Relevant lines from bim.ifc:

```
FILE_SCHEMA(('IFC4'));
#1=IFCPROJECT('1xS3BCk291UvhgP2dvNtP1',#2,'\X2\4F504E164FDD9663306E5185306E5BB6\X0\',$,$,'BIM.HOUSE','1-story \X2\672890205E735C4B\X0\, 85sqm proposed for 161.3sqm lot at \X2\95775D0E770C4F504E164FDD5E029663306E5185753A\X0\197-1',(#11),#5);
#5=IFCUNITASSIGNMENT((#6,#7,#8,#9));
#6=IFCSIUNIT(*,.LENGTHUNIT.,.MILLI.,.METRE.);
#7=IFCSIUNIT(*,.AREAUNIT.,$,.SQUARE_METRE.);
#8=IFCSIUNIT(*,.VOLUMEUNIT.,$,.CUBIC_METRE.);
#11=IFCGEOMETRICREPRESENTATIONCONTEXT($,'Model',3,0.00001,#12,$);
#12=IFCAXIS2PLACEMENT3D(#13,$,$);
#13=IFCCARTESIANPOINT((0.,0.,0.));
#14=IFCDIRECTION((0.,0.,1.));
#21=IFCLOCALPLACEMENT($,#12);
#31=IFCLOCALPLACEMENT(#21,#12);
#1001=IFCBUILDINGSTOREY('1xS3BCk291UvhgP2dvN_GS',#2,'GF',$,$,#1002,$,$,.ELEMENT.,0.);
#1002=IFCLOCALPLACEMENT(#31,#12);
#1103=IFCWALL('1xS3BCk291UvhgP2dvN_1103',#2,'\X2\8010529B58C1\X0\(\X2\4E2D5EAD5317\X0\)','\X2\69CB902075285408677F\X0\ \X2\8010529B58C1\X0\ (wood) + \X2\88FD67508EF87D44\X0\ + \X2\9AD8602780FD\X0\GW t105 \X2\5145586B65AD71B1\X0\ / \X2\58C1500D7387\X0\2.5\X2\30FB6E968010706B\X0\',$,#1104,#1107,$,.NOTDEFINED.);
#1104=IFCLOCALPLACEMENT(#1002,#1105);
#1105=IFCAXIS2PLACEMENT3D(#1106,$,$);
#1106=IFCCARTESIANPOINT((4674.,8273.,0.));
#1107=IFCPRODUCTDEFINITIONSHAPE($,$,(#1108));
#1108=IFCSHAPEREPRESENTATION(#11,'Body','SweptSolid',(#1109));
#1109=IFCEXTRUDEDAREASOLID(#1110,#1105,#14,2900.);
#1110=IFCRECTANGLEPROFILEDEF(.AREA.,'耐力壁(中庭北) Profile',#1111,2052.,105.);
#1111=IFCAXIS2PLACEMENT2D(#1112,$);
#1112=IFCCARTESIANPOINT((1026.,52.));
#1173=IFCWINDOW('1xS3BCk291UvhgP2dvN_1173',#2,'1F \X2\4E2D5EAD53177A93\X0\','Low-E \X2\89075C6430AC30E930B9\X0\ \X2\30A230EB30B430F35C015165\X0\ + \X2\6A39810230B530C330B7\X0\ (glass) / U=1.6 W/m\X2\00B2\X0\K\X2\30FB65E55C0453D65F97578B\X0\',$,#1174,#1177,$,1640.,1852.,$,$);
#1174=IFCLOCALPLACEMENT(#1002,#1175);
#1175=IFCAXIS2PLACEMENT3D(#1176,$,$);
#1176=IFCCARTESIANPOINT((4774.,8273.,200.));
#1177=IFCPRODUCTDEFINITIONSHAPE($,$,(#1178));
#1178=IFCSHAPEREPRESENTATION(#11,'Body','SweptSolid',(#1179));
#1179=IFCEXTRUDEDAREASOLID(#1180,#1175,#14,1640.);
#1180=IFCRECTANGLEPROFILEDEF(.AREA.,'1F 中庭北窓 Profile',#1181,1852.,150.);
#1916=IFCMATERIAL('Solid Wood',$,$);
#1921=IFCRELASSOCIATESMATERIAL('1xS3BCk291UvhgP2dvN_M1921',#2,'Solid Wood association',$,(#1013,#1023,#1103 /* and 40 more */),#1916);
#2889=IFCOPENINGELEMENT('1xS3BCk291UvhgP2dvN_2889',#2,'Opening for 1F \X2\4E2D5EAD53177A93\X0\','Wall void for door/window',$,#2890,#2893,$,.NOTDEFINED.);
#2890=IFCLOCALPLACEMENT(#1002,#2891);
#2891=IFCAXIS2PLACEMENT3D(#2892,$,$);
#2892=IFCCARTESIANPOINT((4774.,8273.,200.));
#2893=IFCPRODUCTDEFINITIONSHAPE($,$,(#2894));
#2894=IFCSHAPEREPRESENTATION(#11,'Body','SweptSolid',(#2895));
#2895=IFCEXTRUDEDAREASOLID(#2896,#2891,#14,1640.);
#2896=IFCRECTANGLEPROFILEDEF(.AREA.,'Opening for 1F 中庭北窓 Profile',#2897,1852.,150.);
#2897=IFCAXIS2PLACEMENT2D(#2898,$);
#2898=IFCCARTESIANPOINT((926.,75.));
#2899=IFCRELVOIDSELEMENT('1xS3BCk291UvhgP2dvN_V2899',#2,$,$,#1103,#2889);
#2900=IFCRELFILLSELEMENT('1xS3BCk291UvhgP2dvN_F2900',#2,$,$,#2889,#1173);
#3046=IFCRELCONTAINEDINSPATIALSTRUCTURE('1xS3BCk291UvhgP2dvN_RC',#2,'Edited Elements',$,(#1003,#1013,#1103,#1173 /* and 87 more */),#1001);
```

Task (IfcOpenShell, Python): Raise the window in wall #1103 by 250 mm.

```python
import numpy as np
import ifcopenshell
import ifcopenshell.api.geometry
import ifcopenshell.util.placement
import ifcopenshell.util.unit

model = ifcopenshell.open("bim.ifc")
unit_scale = ifcopenshell.util.unit.calculate_unit_scale(model)

window = model.by_guid("1xS3BCk291UvhgP2dvN_1173")
opening = window.FillsVoids[0].RelatingOpeningElement
dz = 250.0

shift = np.array([0.0, 0.0, dz])
# The window is not placed relative to its opening, so move both.
for product in (opening, window):
    matrix = ifcopenshell.util.placement.get_local_placement(product.ObjectPlacement)
    matrix[:3, 3] += shift
    ifcopenshell.api.geometry.edit_object_placement(model, product=product, matrix=matrix, is_si=False)

print(f"moved by {dz * unit_scale:+.3f} m")

model.write("bim_edited.ifc")
```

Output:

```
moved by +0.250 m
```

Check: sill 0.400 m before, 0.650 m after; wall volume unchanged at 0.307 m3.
